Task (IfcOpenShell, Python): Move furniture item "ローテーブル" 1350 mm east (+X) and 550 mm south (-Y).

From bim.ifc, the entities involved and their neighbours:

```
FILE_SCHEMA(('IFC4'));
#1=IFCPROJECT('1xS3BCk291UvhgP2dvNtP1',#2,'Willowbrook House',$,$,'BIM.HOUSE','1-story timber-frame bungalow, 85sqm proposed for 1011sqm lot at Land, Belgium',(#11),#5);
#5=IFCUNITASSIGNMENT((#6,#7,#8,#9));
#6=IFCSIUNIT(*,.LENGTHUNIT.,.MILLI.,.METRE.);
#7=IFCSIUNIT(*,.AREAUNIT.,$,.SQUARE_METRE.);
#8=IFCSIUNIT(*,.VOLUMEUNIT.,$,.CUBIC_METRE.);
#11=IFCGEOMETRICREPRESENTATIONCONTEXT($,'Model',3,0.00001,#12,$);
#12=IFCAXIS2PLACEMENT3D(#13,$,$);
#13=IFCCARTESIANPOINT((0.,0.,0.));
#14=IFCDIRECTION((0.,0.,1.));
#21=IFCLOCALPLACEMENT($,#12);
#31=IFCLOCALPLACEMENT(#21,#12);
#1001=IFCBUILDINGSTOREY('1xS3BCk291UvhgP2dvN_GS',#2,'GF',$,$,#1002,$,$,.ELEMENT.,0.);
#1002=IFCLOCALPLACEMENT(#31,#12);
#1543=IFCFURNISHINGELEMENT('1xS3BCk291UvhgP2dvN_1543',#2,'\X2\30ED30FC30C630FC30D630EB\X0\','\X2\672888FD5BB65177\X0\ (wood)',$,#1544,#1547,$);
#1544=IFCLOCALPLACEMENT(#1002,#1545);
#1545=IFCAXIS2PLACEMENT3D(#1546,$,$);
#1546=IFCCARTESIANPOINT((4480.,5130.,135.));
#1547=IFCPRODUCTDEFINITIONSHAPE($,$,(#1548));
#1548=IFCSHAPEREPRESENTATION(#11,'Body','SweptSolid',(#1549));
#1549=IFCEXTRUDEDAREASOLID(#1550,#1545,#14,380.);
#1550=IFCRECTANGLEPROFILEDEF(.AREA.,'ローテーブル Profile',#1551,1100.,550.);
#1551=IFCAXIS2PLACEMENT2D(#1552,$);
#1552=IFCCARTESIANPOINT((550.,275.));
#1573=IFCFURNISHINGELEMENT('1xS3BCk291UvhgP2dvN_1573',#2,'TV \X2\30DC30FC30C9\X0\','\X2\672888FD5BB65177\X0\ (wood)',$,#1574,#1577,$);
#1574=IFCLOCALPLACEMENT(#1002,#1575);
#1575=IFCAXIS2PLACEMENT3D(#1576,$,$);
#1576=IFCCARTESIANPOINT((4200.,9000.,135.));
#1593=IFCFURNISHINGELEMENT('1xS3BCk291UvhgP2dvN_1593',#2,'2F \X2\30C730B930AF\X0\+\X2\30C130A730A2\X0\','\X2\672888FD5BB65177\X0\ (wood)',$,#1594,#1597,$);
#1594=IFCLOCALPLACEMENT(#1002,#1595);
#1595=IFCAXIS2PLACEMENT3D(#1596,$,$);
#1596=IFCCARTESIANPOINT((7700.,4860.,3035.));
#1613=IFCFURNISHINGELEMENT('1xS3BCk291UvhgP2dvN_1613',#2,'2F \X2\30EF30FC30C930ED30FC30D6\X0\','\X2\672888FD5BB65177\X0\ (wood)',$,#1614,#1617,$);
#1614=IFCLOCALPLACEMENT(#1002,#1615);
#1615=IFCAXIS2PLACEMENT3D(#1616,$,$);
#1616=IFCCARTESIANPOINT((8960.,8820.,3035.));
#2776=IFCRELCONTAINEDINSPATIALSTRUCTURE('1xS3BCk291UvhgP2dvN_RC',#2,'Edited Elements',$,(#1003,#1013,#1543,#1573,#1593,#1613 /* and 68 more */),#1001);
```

```python
import ifcopenshell
import ifcopenshell.api.geometry
import ifcopenshell.util.placement
import ifcopenshell.util.unit

model = ifcopenshell.open("bim.ifc")
unit_scale = ifcopenshell.util.unit.calculate_unit_scale(model)

item = model.by_id(1543)
matrix = ifcopenshell.util.placement.get_local_placement(item.ObjectPlacement)
matrix[0, 3] += 1.35 / unit_scale
matrix[1, 3] -= 0.55 / unit_scale
ifcopenshell.api.geometry.edit_object_placement(model, product=item, matrix=matrix, is_si=False)

print(ifcopenshell.util.placement.get_local_placement(item.ObjectPlacement).round(3) + 0.0)

model.write("bim-out.ifc")
```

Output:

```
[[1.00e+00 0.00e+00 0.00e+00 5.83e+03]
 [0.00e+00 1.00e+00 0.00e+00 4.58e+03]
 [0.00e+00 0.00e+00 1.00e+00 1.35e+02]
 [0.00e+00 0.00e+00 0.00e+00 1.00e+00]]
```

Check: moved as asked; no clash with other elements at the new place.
